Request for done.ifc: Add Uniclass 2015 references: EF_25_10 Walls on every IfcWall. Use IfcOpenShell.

First a look at what the model holds.

```python
import ifcopenshell

model = ifcopenshell.open("done.ifc")
print(model.schema)
print("classifications:", [c.Name for c in model.by_type("IfcClassification")])
for ifc_class in ("IfcDoor", "IfcRoof", "IfcStair", "IfcWall", "IfcWindow"):
    print(ifc_class, len(model.by_type(ifc_class)))
```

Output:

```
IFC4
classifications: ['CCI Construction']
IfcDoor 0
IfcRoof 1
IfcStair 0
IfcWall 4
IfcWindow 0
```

```python
import ifcopenshell
import ifcopenshell.api.classification

model = ifcopenshell.open("done.ifc")

system = ifcopenshell.api.classification.add_classification(model, classification="Uniclass 2015")

codes = {
    "IfcWall": ("EF_25_10", "Walls"),
}
for ifc_class, (code, name) in codes.items():
    products = model.by_type(ifc_class)
    ifcopenshell.api.classification.add_reference(
        model, products=products, classification=system, identification=code, name=name
    )
    print(code, len(products))

model.write("done_v2.ifc")
```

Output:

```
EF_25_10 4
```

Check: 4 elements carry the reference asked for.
